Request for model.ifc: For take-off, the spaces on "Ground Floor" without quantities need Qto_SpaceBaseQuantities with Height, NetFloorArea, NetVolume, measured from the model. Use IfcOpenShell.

First a look at what the model holds.

```python
import ifcopenshell
import ifcopenshell.util.element
import ifcopenshell.util.unit

model = ifcopenshell.open("model.ifc")
print(model.schema)
for unit_type in ("LENGTHUNIT", "AREAUNIT", "VOLUMEUNIT"):
    print(unit_type, ifcopenshell.util.unit.calculate_unit_scale(model, unit_type))
storey = next(s for s in model.by_type("IfcBuildingStorey") if s.Name == "Ground Floor")
spaces = [e for e in ifcopenshell.util.element.get_decomposition(storey) if e.is_a("IfcSpace")]
for e in sorted(spaces, key=lambda e: e.id()):
    print(e.id(), e.is_a(), e.Name, list(ifcopenshell.util.element.get_psets(e, qtos_only=True)), sep=" | ")
```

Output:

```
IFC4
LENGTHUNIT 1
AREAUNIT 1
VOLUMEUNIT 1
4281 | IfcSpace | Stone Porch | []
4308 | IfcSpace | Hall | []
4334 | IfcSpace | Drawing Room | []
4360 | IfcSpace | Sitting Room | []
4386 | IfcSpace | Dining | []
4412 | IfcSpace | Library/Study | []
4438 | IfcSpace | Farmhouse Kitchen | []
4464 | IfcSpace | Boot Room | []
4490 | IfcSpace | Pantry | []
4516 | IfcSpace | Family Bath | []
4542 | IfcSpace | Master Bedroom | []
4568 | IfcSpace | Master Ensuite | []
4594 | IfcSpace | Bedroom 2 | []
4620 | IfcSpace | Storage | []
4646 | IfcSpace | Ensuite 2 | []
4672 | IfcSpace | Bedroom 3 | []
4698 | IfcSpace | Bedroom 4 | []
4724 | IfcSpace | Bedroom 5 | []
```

```python
import ifcopenshell
import ifcopenshell.api.pset
import ifcopenshell.geom
import ifcopenshell.util.element
import ifcopenshell.util.shape
import ifcopenshell.util.unit

model = ifcopenshell.open("model.ifc")
unit_scale = ifcopenshell.util.unit.calculate_unit_scale(model)
area_scale = ifcopenshell.util.unit.calculate_unit_scale(model, "AREAUNIT")
volume_scale = ifcopenshell.util.unit.calculate_unit_scale(model, "VOLUMEUNIT")
settings = ifcopenshell.geom.settings()

storey = next(s for s in model.by_type("IfcBuildingStorey") if s.Name == "Ground Floor")
spaces = [e for e in ifcopenshell.util.element.get_decomposition(storey) if e.is_a("IfcSpace")]

for e in sorted(spaces, key=lambda e: e.id()):
    if ifcopenshell.util.element.get_psets(e, qtos_only=True, should_inherit=False):
        continue
    # Geometry comes back in metres, in the element's own axes.
    shape = ifcopenshell.geom.create_shape(settings, e)
    values = {
        "Height": ifcopenshell.util.shape.get_z(shape.geometry) / unit_scale,
        "NetFloorArea": ifcopenshell.util.shape.get_footprint_area(shape.geometry) / area_scale,
        "NetVolume": ifcopenshell.util.shape.get_volume(shape.geometry) / volume_scale,
    }
    qto = ifcopenshell.api.pset.add_qto(model, product=e, name="Qto_SpaceBaseQuantities")
    ifcopenshell.api.pset.edit_qto(model, qto=qto, properties=values)
    print(e.id(), {k: round(v, 3) for k, v in values.items()})

model.write("model_rev.ifc")
```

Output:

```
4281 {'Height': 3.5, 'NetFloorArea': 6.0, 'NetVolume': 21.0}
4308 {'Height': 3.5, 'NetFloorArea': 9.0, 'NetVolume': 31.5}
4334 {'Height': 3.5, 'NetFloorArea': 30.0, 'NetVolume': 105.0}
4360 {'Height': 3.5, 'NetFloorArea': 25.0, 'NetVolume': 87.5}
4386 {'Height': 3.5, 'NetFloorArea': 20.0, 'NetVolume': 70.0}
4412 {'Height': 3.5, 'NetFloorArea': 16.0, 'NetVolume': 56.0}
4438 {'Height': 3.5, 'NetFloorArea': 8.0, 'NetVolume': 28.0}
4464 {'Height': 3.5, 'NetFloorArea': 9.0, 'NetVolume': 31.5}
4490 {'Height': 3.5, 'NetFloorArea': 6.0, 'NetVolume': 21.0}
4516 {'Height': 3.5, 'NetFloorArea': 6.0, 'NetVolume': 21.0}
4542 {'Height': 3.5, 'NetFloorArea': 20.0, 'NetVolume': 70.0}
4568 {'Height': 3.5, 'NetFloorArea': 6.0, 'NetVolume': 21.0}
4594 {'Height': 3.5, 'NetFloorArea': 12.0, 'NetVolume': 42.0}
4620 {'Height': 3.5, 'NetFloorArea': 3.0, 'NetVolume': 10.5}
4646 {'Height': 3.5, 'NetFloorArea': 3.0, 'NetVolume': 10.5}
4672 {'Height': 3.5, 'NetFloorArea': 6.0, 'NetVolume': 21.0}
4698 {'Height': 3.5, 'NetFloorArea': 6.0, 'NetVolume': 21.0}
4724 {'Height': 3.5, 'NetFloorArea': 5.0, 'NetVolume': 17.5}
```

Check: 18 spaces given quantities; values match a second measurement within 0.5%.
